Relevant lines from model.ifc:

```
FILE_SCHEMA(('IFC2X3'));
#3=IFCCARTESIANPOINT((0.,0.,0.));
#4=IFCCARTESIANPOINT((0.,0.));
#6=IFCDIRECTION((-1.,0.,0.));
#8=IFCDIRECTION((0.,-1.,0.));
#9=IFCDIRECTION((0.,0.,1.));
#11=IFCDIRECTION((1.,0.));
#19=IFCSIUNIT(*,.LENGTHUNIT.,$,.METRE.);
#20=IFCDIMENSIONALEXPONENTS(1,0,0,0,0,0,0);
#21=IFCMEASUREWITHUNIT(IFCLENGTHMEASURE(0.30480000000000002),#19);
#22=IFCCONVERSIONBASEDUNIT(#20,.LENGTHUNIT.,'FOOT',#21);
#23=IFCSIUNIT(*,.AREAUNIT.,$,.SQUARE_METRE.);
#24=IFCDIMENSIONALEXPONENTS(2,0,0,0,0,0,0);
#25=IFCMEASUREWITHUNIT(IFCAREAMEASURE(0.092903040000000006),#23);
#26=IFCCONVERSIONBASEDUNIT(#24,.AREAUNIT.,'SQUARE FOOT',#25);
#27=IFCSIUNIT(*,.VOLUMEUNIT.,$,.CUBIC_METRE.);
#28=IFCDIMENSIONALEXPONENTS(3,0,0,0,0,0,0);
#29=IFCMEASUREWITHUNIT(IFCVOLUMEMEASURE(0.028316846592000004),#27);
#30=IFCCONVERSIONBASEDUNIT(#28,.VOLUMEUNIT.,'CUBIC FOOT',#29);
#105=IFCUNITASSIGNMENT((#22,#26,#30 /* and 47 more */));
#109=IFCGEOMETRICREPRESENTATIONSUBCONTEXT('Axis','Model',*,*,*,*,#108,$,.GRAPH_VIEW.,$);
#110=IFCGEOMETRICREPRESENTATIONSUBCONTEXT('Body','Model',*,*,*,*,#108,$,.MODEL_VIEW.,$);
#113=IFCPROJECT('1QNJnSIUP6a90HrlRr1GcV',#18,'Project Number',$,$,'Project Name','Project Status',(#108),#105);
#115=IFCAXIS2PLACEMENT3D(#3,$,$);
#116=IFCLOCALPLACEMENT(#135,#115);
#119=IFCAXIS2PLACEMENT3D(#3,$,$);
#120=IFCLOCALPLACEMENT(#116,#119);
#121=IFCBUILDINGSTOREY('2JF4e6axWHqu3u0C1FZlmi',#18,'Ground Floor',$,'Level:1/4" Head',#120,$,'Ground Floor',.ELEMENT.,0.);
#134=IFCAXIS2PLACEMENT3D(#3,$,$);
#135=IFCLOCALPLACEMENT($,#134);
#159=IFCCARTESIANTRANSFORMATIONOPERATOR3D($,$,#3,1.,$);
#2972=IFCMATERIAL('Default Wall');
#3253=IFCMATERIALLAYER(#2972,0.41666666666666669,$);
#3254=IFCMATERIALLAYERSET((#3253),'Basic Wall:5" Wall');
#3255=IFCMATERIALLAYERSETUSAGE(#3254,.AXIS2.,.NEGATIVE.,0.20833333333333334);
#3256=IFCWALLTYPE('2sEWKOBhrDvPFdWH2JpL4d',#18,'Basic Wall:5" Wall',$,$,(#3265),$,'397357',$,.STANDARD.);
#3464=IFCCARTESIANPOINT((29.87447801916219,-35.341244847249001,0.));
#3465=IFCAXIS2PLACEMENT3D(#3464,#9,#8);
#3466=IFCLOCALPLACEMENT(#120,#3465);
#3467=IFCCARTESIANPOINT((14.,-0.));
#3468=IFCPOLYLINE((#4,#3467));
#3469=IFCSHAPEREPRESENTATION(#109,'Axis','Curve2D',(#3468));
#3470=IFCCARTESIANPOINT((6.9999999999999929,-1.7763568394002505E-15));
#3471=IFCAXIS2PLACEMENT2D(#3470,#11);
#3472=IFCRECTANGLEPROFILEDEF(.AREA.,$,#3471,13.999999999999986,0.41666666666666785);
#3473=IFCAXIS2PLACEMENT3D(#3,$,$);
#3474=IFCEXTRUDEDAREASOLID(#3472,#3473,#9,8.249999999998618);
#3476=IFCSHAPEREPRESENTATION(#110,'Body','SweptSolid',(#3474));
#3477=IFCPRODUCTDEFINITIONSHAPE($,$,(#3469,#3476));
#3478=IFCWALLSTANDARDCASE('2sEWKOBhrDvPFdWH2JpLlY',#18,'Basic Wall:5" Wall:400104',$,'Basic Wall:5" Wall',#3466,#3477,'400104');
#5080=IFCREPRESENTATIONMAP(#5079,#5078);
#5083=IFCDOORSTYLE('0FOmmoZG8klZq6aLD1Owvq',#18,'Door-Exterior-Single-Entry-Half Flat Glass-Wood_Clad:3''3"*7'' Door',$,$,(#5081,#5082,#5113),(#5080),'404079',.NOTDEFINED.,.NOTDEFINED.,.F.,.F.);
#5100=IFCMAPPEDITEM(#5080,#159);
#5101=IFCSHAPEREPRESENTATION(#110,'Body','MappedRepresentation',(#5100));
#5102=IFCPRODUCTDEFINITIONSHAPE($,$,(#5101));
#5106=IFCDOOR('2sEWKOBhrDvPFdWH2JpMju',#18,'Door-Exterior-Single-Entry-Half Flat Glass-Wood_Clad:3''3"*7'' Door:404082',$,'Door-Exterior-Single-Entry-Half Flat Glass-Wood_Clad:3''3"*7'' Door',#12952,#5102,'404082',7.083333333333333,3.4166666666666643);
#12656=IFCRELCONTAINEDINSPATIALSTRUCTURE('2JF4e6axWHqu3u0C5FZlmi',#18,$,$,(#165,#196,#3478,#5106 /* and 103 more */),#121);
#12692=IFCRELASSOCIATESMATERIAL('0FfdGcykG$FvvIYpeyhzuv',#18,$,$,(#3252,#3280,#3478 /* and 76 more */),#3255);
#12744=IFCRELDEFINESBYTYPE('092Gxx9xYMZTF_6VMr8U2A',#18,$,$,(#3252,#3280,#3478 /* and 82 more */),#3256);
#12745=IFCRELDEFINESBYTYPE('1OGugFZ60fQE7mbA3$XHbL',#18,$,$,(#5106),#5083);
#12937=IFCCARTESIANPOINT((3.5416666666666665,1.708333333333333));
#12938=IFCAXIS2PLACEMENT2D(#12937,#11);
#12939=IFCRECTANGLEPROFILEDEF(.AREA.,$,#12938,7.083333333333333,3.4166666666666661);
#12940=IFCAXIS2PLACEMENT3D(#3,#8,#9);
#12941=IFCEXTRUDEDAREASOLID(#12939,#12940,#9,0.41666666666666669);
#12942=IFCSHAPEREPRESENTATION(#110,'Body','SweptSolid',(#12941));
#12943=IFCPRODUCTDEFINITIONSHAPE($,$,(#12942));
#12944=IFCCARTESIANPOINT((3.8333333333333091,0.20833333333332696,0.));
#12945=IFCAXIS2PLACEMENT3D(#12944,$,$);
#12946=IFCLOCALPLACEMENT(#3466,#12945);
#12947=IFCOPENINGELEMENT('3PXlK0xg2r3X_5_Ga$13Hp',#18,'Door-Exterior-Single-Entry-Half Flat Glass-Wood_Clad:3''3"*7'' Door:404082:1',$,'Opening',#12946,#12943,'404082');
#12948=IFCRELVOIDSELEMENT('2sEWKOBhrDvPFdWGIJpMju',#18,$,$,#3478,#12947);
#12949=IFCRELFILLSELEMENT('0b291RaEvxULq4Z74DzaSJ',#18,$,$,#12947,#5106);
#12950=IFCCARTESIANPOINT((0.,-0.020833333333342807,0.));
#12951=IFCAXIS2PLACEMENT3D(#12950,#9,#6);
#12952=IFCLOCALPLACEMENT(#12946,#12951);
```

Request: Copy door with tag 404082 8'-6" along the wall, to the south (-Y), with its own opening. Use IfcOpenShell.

```python
import ifcopenshell
import ifcopenshell.api.feature
import ifcopenshell.api.geometry
import ifcopenshell.api.root
import ifcopenshell.geom
import ifcopenshell.util.element
import ifcopenshell.util.placement
import ifcopenshell.util.shape
import ifcopenshell.util.unit

model = ifcopenshell.open("model.ifc")
unit_scale = ifcopenshell.util.unit.calculate_unit_scale(model)
settings = ifcopenshell.geom.settings()


def volume(element):
    """Net volume in cubic metres, openings subtracted."""
    shape = ifcopenshell.geom.create_shape(settings, element)
    return ifcopenshell.util.shape.get_volume(shape.geometry)


def reuse_history(source, copy):
    """copy_class also copies each property set's owner history, people and application; keep the originals."""
    for rel in copy.IsDefinedBy:
        if rel.is_a("IfcRelDefinesByProperties") and (history := rel.RelatingPropertyDefinition.OwnerHistory):
            rel.RelatingPropertyDefinition.OwnerHistory = source.OwnerHistory
            ifcopenshell.util.element.remove_deep2(model, history)


door = model.by_id(5106)
opening = door.FillsVoids[0].RelatingOpeningElement
wall = opening.VoidsElements[0].RelatingBuildingElement
before = volume(wall)
shift = ifcopenshell.util.placement.get_local_placement(wall.ObjectPlacement)[:3, 0] * 102 * 0.0254 / unit_scale

# copy_class copies the void relationship, type, container and properties, but no geometry.
new_opening = ifcopenshell.api.root.copy_class(model, product=opening)
new_opening.Representation = ifcopenshell.util.element.copy_deep(
    model, opening.Representation, exclude=["IfcGeometricRepresentationContext", "IfcRepresentationMap"]
)
new_opening.Name = 'Door-Exterior-Single-Entry-Half Flat Glass-Wood_Clad:3\'3"*7\' Door'
new_opening.Tag = None
new_door = ifcopenshell.api.root.copy_class(model, product=door)
new_door.Representation = ifcopenshell.util.element.copy_deep(
    model, door.Representation, exclude=["IfcGeometricRepresentationContext", "IfcRepresentationMap"]
)
new_door.Name = 'Door-Exterior-Single-Entry-Half Flat Glass-Wood_Clad:3\'3"*7\' Door'
new_door.Tag = None
reuse_history(door, new_door)
fills = ifcopenshell.api.feature.add_filling(model, opening=new_opening, element=new_door)
fills.OwnerHistory = new_door.OwnerHistory  # required in IFC2X3

for old, new in ((opening, new_opening), (door, new_door)):
    matrix = ifcopenshell.util.placement.get_local_placement(old.ObjectPlacement)
    matrix[:3, 3] += shift
    ifcopenshell.api.geometry.edit_object_placement(model, product=new, matrix=matrix, is_si=False)

after = volume(wall)

print(f"wall volume {before:.3f} -> {after:.3f} m3")

model.write("model-out.ifc")
```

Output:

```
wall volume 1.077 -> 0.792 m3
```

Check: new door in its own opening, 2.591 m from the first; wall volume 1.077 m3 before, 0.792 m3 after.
